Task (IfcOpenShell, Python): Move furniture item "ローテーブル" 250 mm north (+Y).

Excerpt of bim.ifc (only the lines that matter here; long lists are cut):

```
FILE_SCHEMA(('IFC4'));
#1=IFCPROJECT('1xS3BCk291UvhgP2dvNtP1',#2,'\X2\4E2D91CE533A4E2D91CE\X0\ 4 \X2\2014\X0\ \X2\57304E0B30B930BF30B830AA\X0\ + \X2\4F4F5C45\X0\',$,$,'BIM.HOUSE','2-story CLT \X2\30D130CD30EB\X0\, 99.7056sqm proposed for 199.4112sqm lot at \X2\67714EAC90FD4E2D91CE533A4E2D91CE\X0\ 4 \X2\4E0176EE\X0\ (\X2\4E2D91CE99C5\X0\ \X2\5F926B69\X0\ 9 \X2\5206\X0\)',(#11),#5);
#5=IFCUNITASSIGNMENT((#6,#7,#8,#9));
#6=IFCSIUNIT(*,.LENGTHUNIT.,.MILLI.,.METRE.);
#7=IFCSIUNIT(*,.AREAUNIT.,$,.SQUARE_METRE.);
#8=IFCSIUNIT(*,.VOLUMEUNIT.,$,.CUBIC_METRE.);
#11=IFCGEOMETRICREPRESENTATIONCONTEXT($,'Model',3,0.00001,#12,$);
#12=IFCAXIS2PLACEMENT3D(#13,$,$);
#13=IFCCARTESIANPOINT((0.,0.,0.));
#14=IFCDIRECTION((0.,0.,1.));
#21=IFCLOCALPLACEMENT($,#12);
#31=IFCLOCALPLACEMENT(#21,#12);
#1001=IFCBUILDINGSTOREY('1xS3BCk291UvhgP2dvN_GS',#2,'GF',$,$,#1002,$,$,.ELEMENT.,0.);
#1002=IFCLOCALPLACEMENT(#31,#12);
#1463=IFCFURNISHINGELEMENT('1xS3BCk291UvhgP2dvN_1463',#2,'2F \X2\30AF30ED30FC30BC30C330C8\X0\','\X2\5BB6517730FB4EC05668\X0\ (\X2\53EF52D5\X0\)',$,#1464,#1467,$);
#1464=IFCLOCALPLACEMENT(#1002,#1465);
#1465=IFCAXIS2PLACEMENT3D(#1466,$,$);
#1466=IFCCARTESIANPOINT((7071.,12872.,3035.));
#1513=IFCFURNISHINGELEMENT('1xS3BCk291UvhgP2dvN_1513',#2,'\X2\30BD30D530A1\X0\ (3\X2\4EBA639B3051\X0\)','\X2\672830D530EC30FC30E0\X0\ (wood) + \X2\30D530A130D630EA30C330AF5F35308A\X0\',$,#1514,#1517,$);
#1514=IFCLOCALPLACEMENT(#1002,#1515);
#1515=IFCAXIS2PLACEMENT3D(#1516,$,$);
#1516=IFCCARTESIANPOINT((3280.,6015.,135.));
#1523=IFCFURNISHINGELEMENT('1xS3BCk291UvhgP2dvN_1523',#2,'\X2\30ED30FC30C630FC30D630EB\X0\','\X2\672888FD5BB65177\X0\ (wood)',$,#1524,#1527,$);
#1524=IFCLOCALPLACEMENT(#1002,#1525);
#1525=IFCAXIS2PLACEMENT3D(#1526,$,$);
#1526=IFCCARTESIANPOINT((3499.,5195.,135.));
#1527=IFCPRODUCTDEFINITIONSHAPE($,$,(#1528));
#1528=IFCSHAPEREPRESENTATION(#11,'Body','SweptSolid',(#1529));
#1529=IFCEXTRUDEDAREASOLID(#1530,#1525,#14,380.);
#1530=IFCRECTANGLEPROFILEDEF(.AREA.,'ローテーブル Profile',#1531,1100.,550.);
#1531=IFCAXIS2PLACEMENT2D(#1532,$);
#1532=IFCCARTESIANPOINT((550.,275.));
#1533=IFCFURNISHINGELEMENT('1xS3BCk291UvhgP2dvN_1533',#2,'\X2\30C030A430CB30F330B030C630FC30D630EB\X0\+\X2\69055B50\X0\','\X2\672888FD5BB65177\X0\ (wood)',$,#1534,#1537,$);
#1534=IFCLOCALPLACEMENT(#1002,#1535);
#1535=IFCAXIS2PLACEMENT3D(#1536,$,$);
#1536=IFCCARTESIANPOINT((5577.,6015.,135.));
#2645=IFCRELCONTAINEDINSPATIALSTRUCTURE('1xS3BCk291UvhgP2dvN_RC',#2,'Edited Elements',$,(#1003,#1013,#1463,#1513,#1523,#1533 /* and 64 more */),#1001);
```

```python
import ifcopenshell
import ifcopenshell.api.geometry
import ifcopenshell.util.placement
import ifcopenshell.util.unit

model = ifcopenshell.open("bim.ifc")
unit_scale = ifcopenshell.util.unit.calculate_unit_scale(model)

item = model.by_guid("1xS3BCk291UvhgP2dvN_1523")
matrix = ifcopenshell.util.placement.get_local_placement(item.ObjectPlacement)
matrix[1, 3] += 0.25 / unit_scale
ifcopenshell.api.geometry.edit_object_placement(model, product=item, matrix=matrix, is_si=False)

print(ifcopenshell.util.placement.get_local_placement(item.ObjectPlacement).round(3) + 0.0)

model.write("bim_rev.ifc")
```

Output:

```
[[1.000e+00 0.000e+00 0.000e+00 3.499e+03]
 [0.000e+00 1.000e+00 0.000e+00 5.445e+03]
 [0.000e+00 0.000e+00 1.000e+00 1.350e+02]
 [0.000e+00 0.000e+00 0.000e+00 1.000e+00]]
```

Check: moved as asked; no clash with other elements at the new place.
